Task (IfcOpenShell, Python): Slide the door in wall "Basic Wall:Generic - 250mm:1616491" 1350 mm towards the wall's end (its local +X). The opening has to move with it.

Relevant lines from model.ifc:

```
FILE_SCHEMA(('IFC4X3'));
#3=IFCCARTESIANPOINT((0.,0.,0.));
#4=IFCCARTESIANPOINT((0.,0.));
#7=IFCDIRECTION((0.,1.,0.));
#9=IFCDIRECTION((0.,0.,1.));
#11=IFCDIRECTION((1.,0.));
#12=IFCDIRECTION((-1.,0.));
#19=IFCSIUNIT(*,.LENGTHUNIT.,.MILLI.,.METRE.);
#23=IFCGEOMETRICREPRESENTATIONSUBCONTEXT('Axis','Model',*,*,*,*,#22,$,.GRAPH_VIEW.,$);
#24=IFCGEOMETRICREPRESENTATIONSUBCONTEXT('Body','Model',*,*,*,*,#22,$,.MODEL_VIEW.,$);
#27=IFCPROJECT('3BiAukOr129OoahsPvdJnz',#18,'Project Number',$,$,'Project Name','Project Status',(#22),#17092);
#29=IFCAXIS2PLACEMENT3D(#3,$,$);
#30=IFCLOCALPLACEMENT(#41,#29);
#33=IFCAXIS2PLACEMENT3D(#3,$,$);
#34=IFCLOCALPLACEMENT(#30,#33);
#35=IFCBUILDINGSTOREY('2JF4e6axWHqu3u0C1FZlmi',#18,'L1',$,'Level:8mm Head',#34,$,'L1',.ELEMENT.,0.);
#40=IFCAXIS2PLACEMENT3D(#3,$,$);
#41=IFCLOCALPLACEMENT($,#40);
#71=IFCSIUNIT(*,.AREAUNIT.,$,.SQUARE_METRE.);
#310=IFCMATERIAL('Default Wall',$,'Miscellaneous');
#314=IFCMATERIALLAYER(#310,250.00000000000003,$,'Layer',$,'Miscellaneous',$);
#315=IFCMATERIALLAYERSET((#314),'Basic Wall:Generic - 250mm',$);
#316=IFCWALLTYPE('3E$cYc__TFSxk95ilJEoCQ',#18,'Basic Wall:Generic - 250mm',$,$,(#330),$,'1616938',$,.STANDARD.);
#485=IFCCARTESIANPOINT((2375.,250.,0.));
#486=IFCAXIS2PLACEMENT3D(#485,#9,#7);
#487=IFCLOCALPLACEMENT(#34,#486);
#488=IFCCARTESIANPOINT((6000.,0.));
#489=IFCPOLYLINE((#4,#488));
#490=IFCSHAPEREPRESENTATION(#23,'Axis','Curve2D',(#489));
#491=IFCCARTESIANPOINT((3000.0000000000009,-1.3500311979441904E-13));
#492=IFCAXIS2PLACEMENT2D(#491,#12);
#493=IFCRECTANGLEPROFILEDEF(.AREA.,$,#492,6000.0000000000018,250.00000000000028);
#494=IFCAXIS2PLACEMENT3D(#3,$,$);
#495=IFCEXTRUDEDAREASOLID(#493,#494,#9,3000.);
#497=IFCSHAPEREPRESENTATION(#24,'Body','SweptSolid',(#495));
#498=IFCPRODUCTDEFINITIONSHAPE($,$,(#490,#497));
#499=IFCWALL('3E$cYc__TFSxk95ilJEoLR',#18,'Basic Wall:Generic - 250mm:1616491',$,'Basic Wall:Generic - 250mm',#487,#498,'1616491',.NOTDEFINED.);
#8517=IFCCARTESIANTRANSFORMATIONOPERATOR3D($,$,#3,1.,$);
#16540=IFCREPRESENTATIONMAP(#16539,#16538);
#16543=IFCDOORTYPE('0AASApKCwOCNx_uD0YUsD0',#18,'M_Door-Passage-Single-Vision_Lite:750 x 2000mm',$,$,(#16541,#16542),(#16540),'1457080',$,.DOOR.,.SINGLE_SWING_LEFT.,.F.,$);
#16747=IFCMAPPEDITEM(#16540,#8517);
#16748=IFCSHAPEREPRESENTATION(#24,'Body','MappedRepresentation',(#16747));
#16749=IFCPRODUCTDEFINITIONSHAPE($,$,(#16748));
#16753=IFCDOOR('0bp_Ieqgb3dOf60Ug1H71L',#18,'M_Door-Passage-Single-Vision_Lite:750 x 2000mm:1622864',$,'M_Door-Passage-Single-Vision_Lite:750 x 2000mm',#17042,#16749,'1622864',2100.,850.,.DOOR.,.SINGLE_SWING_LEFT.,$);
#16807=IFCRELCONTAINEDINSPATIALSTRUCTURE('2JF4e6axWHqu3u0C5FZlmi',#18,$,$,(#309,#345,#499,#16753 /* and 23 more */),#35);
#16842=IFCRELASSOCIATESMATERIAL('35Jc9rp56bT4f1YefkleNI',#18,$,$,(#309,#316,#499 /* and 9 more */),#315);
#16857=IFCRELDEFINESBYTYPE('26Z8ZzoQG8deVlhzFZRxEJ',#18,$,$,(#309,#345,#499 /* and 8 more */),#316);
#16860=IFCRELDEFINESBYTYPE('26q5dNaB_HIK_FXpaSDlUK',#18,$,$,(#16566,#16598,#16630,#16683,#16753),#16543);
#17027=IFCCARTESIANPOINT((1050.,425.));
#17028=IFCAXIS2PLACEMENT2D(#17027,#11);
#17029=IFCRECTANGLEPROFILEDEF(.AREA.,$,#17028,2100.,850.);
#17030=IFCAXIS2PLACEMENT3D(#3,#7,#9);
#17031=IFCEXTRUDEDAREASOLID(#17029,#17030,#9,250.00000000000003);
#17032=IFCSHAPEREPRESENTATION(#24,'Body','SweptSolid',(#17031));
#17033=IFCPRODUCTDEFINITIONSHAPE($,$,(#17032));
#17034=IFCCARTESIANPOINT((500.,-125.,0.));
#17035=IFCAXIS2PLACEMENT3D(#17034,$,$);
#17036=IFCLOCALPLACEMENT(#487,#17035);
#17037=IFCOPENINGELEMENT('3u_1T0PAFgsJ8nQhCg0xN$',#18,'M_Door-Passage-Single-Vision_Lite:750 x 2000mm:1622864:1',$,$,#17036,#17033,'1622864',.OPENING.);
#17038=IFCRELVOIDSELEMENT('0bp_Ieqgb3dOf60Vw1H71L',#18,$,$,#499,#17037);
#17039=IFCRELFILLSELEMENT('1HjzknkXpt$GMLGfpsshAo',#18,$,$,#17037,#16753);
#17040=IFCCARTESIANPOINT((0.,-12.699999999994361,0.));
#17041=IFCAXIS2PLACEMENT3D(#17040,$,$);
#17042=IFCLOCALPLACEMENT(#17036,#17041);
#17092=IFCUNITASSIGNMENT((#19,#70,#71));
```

```python
import ifcopenshell
import ifcopenshell.api.geometry
import ifcopenshell.util.placement
import ifcopenshell.util.unit

model = ifcopenshell.open("model.ifc")
unit_scale = ifcopenshell.util.unit.calculate_unit_scale(model)

door = model.by_guid("0bp_Ieqgb3dOf60Ug1H71L")
opening = door.FillsVoids[0].RelatingOpeningElement
wall = opening.VoidsElements[0].RelatingBuildingElement

wall_matrix = ifcopenshell.util.placement.get_local_placement(wall.ObjectPlacement)
shift = wall_matrix[:3, 0] * 1.35 / unit_scale
before = ifcopenshell.util.placement.get_local_placement(door.ObjectPlacement)[:3, 3].copy()

# The door is placed relative to its opening, so it follows when the opening moves.
matrix = ifcopenshell.util.placement.get_local_placement(opening.ObjectPlacement)
matrix[:3, 3] += shift
ifcopenshell.api.geometry.edit_object_placement(
    model, product=opening, matrix=matrix, is_si=False, should_transform_children=True
)

after = ifcopenshell.util.placement.get_local_placement(door.ObjectPlacement)[:3, 3]
print("door moved by", (after - before).round(3) + 0.0)

model.write("model-out.ifc")
```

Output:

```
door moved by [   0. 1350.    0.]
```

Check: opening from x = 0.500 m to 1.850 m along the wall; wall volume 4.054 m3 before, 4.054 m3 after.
